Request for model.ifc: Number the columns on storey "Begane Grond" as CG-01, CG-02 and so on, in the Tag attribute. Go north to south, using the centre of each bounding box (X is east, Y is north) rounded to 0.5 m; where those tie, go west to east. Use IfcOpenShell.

First a look at what the model holds.

```python
import ifcopenshell
import ifcopenshell.util.element
import ifcopenshell.util.placement

model = ifcopenshell.open("model.ifc")
print(model.schema)
storey = next(s for s in model.by_type("IfcBuildingStorey") if s.Name == "Begane Grond")
columns = [e for e in ifcopenshell.util.element.get_decomposition(storey) if e.is_a("IfcColumn")]
for e in sorted(columns, key=lambda e: e.id()):
    origin = ifcopenshell.util.placement.get_local_placement(e.ObjectPlacement)[:3, 3]
    print(e.id(), e.Tag, e.Name, origin.round(2) + 0.0, sep=" | ")
```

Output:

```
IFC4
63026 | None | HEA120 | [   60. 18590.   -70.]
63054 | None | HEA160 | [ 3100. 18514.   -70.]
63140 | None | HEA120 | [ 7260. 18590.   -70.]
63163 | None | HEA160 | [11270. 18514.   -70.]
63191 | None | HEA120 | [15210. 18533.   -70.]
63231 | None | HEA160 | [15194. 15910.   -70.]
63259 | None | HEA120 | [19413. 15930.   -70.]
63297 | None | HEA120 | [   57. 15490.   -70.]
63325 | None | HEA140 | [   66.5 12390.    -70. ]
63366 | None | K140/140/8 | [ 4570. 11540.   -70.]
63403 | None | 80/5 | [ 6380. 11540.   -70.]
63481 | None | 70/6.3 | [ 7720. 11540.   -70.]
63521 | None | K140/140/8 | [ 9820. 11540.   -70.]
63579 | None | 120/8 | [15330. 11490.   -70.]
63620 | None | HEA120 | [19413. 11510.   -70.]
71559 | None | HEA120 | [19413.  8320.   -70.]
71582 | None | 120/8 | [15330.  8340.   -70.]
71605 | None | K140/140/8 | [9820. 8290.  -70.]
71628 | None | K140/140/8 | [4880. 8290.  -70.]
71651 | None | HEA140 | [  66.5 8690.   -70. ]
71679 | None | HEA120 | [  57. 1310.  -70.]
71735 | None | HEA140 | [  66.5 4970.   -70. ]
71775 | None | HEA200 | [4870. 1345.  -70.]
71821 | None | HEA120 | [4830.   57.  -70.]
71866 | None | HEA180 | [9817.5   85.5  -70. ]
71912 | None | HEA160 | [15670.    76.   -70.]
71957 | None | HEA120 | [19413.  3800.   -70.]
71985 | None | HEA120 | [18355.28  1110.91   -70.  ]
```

```python
import ifcopenshell
import ifcopenshell.geom
import ifcopenshell.util.element
import ifcopenshell.util.shape

model = ifcopenshell.open("model.ifc")
settings = ifcopenshell.geom.settings()
settings.set("use-world-coords", True)


def centre(element):
    shape = ifcopenshell.geom.create_shape(settings, element)
    return ifcopenshell.util.shape.get_bbox_centroid(shape.geometry)


storey = next(s for s in model.by_type("IfcBuildingStorey") if s.Name == "Begane Grond")
columns = [e for e in ifcopenshell.util.element.get_decomposition(storey) if e.is_a("IfcColumn")]

# Insertion points can sit at a corner or the storey origin, so sort by the geometry (in metres).
centres = {e: centre(e) for e in columns}
columns.sort(key=lambda e: (-round(centres[e][1] / 0.5), centres[e][0]))

for i, e in enumerate(columns, start=1):
    number = f"CG-{i:02d}"
    e.Tag = number
    print(e.id(), number)

model.write("model_updated.ifc")
```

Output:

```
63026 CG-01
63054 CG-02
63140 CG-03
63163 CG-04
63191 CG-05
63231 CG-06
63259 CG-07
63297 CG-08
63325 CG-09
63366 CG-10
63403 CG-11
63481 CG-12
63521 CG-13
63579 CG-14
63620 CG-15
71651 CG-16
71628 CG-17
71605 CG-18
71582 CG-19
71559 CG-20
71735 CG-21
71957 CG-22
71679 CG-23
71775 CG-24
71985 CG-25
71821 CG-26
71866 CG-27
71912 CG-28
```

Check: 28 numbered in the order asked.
